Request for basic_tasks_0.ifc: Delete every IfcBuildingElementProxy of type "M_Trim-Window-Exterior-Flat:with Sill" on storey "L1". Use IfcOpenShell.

First a look at what the model holds.

```python
import ifcopenshell
import ifcopenshell.util.element

model = ifcopenshell.open("basic_tasks_0.ifc")
print(model.schema)
storey = next(s for s in model.by_type("IfcBuildingStorey") if s.Name == "L1")
proxies = [e for e in ifcopenshell.util.element.get_decomposition(storey) if e.is_a("IfcBuildingElementProxy")]
seen = {}
for e in proxies:
    element_type = ifcopenshell.util.element.get_type(e)
    name = element_type.Name if element_type not in (None, e) else None
    seen[name] = seen.get(name, 0) + 1
for name, count in sorted(seen.items(), key=str):
    print(count, "x", name)
```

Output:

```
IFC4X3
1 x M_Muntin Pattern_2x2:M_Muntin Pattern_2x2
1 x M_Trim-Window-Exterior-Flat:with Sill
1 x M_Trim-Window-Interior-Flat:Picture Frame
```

```python
import ifcopenshell
import ifcopenshell.api.root
import ifcopenshell.util.element

model = ifcopenshell.open("basic_tasks_0.ifc")

storey = next(s for s in model.by_type("IfcBuildingStorey") if s.Name == "L1")
proxies = [e for e in ifcopenshell.util.element.get_decomposition(storey) if e.is_a("IfcBuildingElementProxy")]
targets = [e for e in proxies if (t := ifcopenshell.util.element.get_type(e)) not in (None, e) and t.Name == "M_Trim-Window-Exterior-Flat:with Sill"]

for e in targets:
    ifcopenshell.api.root.remove_product(model, product=e)
print(len(targets), "removed")

model.write("basic_tasks_0_rev.ifc")
```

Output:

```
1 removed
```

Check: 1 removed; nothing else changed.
